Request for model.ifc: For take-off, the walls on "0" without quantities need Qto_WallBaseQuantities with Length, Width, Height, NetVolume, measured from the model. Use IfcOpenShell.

First a look at what the model holds.

```python
import ifcopenshell
import ifcopenshell.util.element
import ifcopenshell.util.unit

model = ifcopenshell.open("model.ifc")
print(model.schema)
for unit_type in ("LENGTHUNIT", "AREAUNIT", "VOLUMEUNIT"):
    print(unit_type, ifcopenshell.util.unit.calculate_unit_scale(model, unit_type))
storey = next(s for s in model.by_type("IfcBuildingStorey") if s.Name == "0")
walls = [e for e in ifcopenshell.util.element.get_decomposition(storey) if e.is_a("IfcWall")]
for e in sorted(walls, key=lambda e: e.id()):
    print(e.id(), e.is_a(), e.Name, list(ifcopenshell.util.element.get_psets(e, qtos_only=True)), sep=" | ")
```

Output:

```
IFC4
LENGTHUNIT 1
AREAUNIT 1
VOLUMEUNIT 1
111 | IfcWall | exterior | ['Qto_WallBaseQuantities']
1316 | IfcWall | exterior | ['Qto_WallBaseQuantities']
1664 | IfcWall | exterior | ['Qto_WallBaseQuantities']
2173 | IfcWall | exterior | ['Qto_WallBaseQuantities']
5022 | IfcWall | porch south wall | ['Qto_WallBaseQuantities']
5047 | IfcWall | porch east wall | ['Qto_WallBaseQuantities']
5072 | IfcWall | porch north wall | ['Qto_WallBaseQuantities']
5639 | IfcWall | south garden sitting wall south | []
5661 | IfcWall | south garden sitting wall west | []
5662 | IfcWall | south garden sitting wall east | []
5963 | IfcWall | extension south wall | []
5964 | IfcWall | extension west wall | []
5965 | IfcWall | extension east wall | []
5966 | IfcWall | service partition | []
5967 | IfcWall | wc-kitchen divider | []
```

```python
import ifcopenshell
import ifcopenshell.api.pset
import ifcopenshell.geom
import ifcopenshell.util.element
import ifcopenshell.util.shape
import ifcopenshell.util.unit

model = ifcopenshell.open("model.ifc")
unit_scale = ifcopenshell.util.unit.calculate_unit_scale(model)
volume_scale = ifcopenshell.util.unit.calculate_unit_scale(model, "VOLUMEUNIT")
settings = ifcopenshell.geom.settings()

storey = next(s for s in model.by_type("IfcBuildingStorey") if s.Name == "0")
walls = [e for e in ifcopenshell.util.element.get_decomposition(storey) if e.is_a("IfcWall")]

for e in sorted(walls, key=lambda e: e.id()):
    if ifcopenshell.util.element.get_psets(e, qtos_only=True, should_inherit=False):
        continue
    # Geometry comes back in metres, in the element's own axes.
    shape = ifcopenshell.geom.create_shape(settings, e)
    values = {
        "Length": ifcopenshell.util.shape.get_x(shape.geometry) / unit_scale,
        "Width": ifcopenshell.util.shape.get_y(shape.geometry) / unit_scale,
        "Height": ifcopenshell.util.shape.get_z(shape.geometry) / unit_scale,
        "NetVolume": ifcopenshell.util.shape.get_volume(shape.geometry) / volume_scale,
    }
    qto = ifcopenshell.api.pset.add_qto(model, product=e, name="Qto_WallBaseQuantities")
    ifcopenshell.api.pset.edit_qto(model, qto=qto, properties=values)
    print(e.id(), {k: round(v, 3) for k, v in values.items()})

model.write("model_v2.ifc")
```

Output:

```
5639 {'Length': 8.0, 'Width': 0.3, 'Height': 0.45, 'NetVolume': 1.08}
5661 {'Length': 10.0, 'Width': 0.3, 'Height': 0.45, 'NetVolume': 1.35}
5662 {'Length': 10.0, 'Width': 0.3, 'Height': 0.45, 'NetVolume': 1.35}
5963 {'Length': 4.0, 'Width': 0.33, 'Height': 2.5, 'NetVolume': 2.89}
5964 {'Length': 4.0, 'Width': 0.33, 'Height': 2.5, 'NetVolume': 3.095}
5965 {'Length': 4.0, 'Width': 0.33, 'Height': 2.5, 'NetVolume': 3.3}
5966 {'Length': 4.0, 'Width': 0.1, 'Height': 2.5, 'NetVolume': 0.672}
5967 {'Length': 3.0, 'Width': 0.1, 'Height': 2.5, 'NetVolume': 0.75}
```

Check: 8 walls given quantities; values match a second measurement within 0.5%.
